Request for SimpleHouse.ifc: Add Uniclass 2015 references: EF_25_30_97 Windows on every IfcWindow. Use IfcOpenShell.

First a look at what the model holds.

```python
import ifcopenshell

model = ifcopenshell.open("SimpleHouse.ifc")
print(model.schema)
print("classifications:", [c.Name for c in model.by_type("IfcClassification")])
for ifc_class in ("IfcDoor", "IfcRoof", "IfcStair", "IfcWall", "IfcWindow"):
    print(ifc_class, len(model.by_type(ifc_class)))
```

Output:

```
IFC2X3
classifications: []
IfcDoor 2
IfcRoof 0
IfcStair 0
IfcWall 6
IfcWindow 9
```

```python
import ifcopenshell
import ifcopenshell.api.classification

model = ifcopenshell.open("SimpleHouse.ifc")

# IFC2X3 requires Source and Edition and has no link from the project to the system.
system = model.create_entity("IfcClassification", Source="NBS", Edition="2015", Name="Uniclass 2015")

codes = {
    "IfcWindow": ("EF_25_30_97", "Windows"),
}
for ifc_class, (code, name) in codes.items():
    products = model.by_type(ifc_class)
    ifcopenshell.api.classification.add_reference(
        model, products=products, classification=system, identification=code, name=name
    )
    print(code, len(products))

model.write("SimpleHouse_v2.ifc")
```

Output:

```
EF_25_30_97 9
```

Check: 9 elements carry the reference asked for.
